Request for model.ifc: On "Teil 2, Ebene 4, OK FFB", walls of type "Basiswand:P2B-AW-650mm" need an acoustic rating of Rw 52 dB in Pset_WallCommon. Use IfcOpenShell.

First a look at what the model holds.

```python
import ifcopenshell
import ifcopenshell.util.element

model = ifcopenshell.open("model.ifc")
print(model.schema)
storey = next(s for s in model.by_type("IfcBuildingStorey") if s.Name == "Teil 2, Ebene 4, OK FFB")
walls = [e for e in ifcopenshell.util.element.get_decomposition(storey) if e.is_a("IfcWall")]
seen = {}
for e in walls:
    element_type = ifcopenshell.util.element.get_type(e)
    key = (element_type.Name if element_type != e and element_type else None, ifcopenshell.util.element.get_pset(e, "Pset_WallCommon", "AcousticRating"))
    seen[key] = seen.get(key, 0) + 1
for (name, value), count in sorted(seen.items(), key=str):
    print(count, "x", name, "|", value)
```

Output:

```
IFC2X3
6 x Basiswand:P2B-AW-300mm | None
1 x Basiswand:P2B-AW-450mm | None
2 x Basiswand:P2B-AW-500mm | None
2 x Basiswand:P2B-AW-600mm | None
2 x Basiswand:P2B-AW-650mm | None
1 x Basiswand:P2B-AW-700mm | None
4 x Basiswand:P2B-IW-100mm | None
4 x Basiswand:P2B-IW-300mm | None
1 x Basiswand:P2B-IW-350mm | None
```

```python
import ifcopenshell
import ifcopenshell.api.pset
import ifcopenshell.util.element

model = ifcopenshell.open("model.ifc")

storey = next(s for s in model.by_type("IfcBuildingStorey") if s.Name == "Teil 2, Ebene 4, OK FFB")
walls = [e for e in ifcopenshell.util.element.get_decomposition(storey) if e.is_a("IfcWall")]

count = 0
for e in walls:
    element_type = ifcopenshell.util.element.get_type(e)
    if element_type in (None, e) or element_type.Name != "Basiswand:P2B-AW-650mm":
        continue
    # add_pset returns the element's existing set when there is one.
    pset = ifcopenshell.api.pset.add_pset(model, product=e, name="Pset_WallCommon")
    ifcopenshell.api.pset.edit_pset(model, pset=pset, properties={"AcousticRating": "Rw 52 dB"})
    count += 1

print(count, "walls updated")

model.write("model_edited.ifc")
```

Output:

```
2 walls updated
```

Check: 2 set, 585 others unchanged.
